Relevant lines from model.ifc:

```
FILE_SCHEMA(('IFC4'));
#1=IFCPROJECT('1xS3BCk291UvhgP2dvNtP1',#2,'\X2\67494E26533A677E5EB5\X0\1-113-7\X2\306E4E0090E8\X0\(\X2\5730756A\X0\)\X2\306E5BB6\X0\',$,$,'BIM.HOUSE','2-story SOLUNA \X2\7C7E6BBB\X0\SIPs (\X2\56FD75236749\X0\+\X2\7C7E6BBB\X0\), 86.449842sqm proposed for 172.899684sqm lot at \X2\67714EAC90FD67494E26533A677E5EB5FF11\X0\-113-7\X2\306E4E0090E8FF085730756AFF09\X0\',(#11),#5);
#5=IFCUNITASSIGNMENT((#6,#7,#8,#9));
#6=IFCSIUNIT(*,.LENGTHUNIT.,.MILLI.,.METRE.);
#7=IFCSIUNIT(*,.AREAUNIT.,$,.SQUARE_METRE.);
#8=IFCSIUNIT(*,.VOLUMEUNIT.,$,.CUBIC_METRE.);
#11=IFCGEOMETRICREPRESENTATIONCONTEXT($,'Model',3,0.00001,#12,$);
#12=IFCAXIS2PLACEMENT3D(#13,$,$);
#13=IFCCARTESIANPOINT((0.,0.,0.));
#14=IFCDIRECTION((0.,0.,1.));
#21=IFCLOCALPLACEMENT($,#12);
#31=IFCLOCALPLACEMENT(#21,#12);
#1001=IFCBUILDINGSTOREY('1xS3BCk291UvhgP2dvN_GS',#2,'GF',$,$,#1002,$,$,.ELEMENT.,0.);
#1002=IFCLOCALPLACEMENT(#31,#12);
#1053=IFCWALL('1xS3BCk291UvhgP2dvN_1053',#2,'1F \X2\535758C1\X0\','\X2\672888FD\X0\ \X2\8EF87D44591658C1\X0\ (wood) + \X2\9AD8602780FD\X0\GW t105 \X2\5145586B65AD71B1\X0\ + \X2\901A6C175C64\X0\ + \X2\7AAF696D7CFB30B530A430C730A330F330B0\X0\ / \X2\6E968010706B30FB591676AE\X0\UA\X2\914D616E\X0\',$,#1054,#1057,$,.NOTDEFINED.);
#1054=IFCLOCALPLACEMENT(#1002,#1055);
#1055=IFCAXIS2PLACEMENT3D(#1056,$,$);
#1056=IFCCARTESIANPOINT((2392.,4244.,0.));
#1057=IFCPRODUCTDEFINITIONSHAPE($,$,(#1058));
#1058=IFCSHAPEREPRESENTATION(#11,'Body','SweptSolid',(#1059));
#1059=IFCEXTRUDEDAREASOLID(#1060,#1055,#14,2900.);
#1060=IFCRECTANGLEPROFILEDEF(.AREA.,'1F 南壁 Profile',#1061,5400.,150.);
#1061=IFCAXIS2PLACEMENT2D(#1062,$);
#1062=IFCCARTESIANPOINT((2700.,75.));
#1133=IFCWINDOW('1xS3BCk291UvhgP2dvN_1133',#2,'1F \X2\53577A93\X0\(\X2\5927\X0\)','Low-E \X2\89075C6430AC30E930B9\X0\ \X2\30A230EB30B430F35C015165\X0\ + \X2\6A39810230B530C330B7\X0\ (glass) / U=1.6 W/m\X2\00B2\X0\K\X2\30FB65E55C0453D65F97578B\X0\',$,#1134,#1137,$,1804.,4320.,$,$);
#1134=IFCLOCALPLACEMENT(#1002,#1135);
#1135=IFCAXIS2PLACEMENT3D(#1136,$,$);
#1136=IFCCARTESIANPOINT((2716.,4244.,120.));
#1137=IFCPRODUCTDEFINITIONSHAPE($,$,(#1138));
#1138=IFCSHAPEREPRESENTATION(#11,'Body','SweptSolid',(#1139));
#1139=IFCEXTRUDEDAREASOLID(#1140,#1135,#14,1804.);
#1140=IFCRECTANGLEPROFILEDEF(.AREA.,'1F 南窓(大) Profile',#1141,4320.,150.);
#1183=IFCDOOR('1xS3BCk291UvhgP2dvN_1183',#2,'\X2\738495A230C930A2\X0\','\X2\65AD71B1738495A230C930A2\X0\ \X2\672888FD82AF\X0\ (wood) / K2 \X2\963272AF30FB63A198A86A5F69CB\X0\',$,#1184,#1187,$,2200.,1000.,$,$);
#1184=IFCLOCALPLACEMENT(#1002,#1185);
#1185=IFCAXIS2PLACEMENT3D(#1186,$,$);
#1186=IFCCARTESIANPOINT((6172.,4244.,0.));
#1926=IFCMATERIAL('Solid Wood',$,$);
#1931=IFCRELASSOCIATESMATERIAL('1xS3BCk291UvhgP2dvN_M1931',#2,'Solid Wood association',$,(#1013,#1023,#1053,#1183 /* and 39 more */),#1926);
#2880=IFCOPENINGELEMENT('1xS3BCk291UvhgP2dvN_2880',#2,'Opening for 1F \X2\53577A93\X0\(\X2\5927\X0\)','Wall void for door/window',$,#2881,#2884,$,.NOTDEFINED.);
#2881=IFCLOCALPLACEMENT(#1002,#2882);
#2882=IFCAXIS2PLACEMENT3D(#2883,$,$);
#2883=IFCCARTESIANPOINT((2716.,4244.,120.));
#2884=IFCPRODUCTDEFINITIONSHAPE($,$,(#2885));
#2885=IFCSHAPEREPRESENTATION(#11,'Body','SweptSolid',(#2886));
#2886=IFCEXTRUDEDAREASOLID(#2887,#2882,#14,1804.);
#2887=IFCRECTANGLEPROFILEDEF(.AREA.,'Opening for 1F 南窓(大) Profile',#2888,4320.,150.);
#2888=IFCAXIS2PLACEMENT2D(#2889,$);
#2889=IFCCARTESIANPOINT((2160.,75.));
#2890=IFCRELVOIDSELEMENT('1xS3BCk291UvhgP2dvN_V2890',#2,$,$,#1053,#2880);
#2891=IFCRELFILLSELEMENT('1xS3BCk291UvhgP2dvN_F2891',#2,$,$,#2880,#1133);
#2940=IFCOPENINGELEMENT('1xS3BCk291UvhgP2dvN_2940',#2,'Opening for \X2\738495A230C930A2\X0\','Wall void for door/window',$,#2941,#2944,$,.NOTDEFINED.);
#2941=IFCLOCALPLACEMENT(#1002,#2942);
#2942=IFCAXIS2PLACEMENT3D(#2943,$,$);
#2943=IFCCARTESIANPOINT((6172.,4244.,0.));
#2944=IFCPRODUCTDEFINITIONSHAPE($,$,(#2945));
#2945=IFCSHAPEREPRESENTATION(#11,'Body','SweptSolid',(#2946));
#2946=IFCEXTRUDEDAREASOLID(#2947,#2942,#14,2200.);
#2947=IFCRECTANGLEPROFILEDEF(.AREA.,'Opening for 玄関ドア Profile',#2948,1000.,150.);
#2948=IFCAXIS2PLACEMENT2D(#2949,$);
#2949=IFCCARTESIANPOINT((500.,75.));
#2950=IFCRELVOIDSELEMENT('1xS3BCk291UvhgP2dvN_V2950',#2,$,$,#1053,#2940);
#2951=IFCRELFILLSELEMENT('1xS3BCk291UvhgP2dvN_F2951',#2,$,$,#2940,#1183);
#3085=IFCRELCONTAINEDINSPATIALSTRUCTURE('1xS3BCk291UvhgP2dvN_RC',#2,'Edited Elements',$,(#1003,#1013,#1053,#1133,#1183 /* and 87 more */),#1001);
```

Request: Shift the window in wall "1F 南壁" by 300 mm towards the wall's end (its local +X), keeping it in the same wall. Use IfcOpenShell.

```python
import ifcopenshell
import ifcopenshell.api.geometry
import ifcopenshell.util.placement

model = ifcopenshell.open("model.ifc")

window = model.by_id(1133)
opening = window.FillsVoids[0].RelatingOpeningElement
wall = opening.VoidsElements[0].RelatingBuildingElement

wall_matrix = ifcopenshell.util.placement.get_local_placement(wall.ObjectPlacement)
shift = wall_matrix[:3, 0] * 300.0
before = ifcopenshell.util.placement.get_local_placement(window.ObjectPlacement)[:3, 3].copy()

# The window is not placed relative to its opening, so move both.
for product in (opening, window):
    matrix = ifcopenshell.util.placement.get_local_placement(product.ObjectPlacement)
    matrix[:3, 3] += shift
    ifcopenshell.api.geometry.edit_object_placement(model, product=product, matrix=matrix, is_si=False)

after = ifcopenshell.util.placement.get_local_placement(window.ObjectPlacement)[:3, 3]
print("window moved by", (after - before).round(3) + 0.0)

model.write("model_updated.ifc")
```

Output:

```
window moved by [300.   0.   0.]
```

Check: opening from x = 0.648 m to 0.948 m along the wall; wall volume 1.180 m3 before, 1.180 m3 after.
